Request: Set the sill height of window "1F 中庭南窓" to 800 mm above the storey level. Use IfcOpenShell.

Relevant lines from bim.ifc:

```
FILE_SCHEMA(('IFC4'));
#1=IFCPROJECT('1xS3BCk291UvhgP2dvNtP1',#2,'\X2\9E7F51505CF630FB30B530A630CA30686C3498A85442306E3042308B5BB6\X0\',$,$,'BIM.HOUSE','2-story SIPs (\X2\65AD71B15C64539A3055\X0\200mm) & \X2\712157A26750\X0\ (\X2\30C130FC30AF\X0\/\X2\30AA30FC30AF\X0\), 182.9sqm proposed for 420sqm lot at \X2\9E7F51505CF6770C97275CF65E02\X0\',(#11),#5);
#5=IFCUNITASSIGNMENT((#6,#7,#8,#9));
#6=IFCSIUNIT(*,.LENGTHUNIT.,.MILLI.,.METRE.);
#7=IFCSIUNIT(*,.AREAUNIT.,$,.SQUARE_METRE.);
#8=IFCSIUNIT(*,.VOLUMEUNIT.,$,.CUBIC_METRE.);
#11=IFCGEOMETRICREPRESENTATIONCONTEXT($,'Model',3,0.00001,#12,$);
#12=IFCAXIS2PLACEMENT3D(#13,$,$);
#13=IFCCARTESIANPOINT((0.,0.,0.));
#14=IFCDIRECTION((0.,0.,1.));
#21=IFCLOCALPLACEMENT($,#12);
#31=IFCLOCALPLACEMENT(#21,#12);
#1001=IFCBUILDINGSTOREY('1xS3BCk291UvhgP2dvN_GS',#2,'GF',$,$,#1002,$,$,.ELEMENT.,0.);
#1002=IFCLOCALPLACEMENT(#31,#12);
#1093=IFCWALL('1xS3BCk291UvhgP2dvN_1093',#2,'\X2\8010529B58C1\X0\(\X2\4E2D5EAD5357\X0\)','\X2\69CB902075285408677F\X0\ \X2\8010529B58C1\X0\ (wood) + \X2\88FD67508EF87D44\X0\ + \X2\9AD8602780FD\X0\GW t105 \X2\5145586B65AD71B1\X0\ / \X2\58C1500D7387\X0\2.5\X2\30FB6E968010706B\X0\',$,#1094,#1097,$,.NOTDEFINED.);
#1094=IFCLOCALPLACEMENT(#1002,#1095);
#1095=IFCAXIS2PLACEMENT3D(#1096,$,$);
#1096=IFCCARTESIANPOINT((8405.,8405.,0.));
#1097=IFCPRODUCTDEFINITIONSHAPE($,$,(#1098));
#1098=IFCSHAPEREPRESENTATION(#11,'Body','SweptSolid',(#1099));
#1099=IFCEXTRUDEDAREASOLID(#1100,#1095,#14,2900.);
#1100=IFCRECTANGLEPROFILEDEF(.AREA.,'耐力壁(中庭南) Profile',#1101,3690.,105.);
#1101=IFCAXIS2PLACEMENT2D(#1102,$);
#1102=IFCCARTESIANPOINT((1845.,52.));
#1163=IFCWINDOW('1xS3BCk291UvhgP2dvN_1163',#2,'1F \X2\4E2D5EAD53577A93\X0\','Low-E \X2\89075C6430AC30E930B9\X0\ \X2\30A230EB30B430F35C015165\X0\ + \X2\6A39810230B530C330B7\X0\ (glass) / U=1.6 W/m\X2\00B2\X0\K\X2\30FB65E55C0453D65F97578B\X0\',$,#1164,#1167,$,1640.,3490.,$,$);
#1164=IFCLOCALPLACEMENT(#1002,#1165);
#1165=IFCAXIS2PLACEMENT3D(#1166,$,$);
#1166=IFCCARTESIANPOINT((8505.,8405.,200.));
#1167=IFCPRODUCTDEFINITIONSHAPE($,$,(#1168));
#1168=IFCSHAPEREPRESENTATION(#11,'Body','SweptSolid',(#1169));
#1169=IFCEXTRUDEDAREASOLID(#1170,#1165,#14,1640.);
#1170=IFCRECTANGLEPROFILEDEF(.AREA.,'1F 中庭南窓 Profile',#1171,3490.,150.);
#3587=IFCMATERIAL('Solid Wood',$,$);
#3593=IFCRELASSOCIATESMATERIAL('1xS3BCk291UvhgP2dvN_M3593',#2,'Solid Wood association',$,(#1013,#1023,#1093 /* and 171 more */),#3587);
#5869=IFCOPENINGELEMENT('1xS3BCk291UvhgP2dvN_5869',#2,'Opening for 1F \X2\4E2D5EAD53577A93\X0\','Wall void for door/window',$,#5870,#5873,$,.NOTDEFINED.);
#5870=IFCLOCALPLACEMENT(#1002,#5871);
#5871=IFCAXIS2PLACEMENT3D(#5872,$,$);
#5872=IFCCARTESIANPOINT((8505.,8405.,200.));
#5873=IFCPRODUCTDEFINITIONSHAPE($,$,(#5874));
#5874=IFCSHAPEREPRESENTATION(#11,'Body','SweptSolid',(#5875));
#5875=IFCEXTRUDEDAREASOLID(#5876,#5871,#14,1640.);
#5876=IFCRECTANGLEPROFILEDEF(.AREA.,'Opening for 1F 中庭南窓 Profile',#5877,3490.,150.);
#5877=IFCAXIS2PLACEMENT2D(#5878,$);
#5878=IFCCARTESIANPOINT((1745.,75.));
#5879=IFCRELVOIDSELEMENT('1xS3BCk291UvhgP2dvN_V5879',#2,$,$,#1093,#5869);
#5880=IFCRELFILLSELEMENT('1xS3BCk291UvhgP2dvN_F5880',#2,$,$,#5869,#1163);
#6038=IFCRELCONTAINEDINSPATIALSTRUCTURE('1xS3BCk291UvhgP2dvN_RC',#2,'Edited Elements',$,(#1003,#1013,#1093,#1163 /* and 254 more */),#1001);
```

```python
import numpy as np
import ifcopenshell
import ifcopenshell.api.geometry
import ifcopenshell.geom
import ifcopenshell.util.element
import ifcopenshell.util.placement
import ifcopenshell.util.shape
import ifcopenshell.util.unit

model = ifcopenshell.open("bim.ifc")
unit_scale = ifcopenshell.util.unit.calculate_unit_scale(model)

window = model.by_guid("1xS3BCk291UvhgP2dvN_1163")
opening = window.FillsVoids[0].RelatingOpeningElement
storey = ifcopenshell.util.element.get_container(window, ifc_class="IfcBuildingStorey")
level = ifcopenshell.util.placement.get_local_placement(storey.ObjectPlacement)[2, 3]

# The opening's origin need not be at the sill, so measure its lowest point.
shape = ifcopenshell.geom.create_shape(ifcopenshell.geom.settings(), opening)
bottom = ifcopenshell.util.shape.get_shape_bottom_elevation(shape, shape.geometry) / unit_scale
dz = level + 800.0 - bottom

shift = np.array([0.0, 0.0, dz])
# The window is not placed relative to its opening, so move both.
for product in (opening, window):
    matrix = ifcopenshell.util.placement.get_local_placement(product.ObjectPlacement)
    matrix[:3, 3] += shift
    ifcopenshell.api.geometry.edit_object_placement(model, product=product, matrix=matrix, is_si=False)

print(f"moved by {dz * unit_scale:+.3f} m")

model.write("bim_updated.ifc")
```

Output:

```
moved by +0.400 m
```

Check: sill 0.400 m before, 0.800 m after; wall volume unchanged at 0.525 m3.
